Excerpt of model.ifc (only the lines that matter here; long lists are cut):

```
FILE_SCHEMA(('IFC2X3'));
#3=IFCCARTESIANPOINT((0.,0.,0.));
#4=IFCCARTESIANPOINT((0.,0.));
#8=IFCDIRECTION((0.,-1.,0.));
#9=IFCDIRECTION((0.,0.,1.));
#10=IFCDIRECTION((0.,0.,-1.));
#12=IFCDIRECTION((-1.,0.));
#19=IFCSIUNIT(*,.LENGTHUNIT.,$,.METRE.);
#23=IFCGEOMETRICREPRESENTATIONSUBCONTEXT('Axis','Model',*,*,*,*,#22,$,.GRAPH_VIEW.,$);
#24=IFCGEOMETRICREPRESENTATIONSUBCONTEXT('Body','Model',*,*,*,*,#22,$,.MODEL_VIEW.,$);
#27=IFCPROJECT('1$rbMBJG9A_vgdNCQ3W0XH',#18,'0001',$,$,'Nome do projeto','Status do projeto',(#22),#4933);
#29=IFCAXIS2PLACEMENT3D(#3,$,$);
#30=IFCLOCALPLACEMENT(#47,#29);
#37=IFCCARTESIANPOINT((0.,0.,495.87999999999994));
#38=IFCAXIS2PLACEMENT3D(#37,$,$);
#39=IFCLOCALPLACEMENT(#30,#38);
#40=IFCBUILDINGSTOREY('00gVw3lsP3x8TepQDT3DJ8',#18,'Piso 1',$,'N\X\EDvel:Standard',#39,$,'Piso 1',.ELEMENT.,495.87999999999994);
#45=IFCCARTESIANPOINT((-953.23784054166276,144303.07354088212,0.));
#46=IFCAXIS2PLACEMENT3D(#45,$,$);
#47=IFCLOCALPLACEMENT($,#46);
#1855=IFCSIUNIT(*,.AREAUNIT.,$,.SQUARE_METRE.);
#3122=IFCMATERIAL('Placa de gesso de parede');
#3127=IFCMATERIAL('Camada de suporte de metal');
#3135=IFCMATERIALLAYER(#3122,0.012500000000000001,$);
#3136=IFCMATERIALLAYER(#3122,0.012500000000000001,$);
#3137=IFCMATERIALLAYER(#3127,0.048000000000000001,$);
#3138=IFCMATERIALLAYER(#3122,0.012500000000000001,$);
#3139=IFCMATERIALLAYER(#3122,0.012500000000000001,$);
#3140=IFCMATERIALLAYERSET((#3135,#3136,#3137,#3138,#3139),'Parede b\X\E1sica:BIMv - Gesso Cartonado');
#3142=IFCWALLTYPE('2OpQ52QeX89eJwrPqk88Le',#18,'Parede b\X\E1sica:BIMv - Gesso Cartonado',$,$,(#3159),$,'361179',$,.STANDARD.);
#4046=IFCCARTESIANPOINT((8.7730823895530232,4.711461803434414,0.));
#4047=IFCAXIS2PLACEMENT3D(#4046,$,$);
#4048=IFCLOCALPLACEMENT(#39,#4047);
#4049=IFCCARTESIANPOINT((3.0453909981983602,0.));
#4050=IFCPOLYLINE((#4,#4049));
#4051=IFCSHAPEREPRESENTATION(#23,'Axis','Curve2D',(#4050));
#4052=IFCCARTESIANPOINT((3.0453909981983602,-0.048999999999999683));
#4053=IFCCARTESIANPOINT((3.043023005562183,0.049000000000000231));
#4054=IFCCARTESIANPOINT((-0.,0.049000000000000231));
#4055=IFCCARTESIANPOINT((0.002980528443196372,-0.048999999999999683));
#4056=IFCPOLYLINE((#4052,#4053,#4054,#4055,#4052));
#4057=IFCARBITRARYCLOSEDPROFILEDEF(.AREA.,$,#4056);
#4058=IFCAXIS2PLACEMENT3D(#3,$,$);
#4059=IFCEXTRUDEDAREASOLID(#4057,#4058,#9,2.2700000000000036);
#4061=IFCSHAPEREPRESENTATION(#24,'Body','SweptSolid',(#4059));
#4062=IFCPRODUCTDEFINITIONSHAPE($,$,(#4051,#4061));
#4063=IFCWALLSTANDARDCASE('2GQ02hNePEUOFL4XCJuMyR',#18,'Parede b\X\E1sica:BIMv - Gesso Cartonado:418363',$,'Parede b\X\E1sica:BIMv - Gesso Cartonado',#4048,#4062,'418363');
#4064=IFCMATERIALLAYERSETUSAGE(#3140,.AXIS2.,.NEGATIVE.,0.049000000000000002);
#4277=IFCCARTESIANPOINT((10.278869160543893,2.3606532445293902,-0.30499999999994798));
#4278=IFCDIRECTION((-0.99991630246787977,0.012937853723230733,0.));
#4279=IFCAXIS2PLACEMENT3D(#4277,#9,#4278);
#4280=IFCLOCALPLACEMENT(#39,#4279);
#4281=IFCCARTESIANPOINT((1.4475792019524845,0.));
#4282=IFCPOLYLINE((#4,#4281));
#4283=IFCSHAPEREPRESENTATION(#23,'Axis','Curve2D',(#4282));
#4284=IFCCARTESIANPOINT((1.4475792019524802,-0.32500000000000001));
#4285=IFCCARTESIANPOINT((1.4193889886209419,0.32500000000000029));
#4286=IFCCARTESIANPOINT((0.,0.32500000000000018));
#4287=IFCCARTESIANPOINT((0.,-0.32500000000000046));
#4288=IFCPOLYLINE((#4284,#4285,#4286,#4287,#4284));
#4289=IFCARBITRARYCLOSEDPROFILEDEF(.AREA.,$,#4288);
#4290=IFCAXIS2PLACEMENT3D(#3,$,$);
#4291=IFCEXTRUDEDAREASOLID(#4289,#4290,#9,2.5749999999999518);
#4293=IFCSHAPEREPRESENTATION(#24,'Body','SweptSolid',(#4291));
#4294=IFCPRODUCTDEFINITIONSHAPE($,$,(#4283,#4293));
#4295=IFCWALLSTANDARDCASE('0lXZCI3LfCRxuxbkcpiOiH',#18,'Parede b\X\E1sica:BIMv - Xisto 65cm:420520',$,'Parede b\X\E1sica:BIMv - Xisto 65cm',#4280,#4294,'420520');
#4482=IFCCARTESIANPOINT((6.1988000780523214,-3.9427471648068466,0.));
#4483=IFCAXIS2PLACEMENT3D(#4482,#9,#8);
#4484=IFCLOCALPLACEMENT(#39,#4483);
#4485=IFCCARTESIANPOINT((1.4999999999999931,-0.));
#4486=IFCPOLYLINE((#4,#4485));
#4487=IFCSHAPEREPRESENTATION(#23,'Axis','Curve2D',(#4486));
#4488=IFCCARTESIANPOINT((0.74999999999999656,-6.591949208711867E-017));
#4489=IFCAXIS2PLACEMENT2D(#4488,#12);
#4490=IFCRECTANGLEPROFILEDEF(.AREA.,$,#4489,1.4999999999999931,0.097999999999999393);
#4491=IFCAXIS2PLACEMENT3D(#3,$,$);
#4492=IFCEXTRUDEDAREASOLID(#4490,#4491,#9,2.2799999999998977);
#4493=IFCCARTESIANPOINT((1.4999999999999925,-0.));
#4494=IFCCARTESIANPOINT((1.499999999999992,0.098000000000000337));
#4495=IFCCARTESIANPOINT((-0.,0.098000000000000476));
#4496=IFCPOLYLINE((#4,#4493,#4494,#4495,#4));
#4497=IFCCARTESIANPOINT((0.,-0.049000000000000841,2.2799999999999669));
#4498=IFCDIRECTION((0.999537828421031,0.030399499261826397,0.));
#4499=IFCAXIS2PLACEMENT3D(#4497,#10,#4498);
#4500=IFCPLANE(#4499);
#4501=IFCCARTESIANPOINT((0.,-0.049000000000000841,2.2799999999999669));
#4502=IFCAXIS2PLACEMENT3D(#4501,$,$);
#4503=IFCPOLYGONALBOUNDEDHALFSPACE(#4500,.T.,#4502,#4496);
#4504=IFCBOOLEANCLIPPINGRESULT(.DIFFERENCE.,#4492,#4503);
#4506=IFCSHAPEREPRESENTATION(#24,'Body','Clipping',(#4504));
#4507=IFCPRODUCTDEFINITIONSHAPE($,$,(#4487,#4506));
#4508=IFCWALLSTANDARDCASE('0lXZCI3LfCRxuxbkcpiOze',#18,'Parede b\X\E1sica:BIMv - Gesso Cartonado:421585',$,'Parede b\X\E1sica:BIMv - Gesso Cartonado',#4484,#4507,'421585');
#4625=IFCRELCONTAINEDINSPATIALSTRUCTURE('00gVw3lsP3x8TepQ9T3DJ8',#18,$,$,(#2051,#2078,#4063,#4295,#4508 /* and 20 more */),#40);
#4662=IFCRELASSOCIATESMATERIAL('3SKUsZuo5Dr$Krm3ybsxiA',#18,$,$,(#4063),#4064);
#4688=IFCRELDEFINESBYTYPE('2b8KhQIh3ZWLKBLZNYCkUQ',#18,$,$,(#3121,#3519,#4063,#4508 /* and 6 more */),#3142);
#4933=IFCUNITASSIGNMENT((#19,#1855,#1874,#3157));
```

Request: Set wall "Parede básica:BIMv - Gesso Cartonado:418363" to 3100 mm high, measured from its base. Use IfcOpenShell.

```python
import ifcopenshell
import ifcopenshell.geom
import ifcopenshell.util.representation
import ifcopenshell.util.shape
import ifcopenshell.util.unit

model = ifcopenshell.open("model.ifc")
unit_scale = ifcopenshell.util.unit.calculate_unit_scale(model)
settings = ifcopenshell.geom.settings()


def volume(element):
    """Net volume in cubic metres, openings subtracted."""
    shape = ifcopenshell.geom.create_shape(settings, element)
    return ifcopenshell.util.shape.get_volume(shape.geometry)


wall = model.by_guid("2GQ02hNePEUOFL4XCJuMyR")
before = volume(wall)

body = ifcopenshell.util.representation.get_representation(wall, "Model", "Body")
solid = body.Items[0]
old_height = solid.Depth
solid.Depth = 3.1 / unit_scale
after = volume(wall)

print(f"height {old_height:g} -> {solid.Depth:g}, volume {before:.3f} -> {after:.3f} m3")

model.write("model_v2.ifc")
```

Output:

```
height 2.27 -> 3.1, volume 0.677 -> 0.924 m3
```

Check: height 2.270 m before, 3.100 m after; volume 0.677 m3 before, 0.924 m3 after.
